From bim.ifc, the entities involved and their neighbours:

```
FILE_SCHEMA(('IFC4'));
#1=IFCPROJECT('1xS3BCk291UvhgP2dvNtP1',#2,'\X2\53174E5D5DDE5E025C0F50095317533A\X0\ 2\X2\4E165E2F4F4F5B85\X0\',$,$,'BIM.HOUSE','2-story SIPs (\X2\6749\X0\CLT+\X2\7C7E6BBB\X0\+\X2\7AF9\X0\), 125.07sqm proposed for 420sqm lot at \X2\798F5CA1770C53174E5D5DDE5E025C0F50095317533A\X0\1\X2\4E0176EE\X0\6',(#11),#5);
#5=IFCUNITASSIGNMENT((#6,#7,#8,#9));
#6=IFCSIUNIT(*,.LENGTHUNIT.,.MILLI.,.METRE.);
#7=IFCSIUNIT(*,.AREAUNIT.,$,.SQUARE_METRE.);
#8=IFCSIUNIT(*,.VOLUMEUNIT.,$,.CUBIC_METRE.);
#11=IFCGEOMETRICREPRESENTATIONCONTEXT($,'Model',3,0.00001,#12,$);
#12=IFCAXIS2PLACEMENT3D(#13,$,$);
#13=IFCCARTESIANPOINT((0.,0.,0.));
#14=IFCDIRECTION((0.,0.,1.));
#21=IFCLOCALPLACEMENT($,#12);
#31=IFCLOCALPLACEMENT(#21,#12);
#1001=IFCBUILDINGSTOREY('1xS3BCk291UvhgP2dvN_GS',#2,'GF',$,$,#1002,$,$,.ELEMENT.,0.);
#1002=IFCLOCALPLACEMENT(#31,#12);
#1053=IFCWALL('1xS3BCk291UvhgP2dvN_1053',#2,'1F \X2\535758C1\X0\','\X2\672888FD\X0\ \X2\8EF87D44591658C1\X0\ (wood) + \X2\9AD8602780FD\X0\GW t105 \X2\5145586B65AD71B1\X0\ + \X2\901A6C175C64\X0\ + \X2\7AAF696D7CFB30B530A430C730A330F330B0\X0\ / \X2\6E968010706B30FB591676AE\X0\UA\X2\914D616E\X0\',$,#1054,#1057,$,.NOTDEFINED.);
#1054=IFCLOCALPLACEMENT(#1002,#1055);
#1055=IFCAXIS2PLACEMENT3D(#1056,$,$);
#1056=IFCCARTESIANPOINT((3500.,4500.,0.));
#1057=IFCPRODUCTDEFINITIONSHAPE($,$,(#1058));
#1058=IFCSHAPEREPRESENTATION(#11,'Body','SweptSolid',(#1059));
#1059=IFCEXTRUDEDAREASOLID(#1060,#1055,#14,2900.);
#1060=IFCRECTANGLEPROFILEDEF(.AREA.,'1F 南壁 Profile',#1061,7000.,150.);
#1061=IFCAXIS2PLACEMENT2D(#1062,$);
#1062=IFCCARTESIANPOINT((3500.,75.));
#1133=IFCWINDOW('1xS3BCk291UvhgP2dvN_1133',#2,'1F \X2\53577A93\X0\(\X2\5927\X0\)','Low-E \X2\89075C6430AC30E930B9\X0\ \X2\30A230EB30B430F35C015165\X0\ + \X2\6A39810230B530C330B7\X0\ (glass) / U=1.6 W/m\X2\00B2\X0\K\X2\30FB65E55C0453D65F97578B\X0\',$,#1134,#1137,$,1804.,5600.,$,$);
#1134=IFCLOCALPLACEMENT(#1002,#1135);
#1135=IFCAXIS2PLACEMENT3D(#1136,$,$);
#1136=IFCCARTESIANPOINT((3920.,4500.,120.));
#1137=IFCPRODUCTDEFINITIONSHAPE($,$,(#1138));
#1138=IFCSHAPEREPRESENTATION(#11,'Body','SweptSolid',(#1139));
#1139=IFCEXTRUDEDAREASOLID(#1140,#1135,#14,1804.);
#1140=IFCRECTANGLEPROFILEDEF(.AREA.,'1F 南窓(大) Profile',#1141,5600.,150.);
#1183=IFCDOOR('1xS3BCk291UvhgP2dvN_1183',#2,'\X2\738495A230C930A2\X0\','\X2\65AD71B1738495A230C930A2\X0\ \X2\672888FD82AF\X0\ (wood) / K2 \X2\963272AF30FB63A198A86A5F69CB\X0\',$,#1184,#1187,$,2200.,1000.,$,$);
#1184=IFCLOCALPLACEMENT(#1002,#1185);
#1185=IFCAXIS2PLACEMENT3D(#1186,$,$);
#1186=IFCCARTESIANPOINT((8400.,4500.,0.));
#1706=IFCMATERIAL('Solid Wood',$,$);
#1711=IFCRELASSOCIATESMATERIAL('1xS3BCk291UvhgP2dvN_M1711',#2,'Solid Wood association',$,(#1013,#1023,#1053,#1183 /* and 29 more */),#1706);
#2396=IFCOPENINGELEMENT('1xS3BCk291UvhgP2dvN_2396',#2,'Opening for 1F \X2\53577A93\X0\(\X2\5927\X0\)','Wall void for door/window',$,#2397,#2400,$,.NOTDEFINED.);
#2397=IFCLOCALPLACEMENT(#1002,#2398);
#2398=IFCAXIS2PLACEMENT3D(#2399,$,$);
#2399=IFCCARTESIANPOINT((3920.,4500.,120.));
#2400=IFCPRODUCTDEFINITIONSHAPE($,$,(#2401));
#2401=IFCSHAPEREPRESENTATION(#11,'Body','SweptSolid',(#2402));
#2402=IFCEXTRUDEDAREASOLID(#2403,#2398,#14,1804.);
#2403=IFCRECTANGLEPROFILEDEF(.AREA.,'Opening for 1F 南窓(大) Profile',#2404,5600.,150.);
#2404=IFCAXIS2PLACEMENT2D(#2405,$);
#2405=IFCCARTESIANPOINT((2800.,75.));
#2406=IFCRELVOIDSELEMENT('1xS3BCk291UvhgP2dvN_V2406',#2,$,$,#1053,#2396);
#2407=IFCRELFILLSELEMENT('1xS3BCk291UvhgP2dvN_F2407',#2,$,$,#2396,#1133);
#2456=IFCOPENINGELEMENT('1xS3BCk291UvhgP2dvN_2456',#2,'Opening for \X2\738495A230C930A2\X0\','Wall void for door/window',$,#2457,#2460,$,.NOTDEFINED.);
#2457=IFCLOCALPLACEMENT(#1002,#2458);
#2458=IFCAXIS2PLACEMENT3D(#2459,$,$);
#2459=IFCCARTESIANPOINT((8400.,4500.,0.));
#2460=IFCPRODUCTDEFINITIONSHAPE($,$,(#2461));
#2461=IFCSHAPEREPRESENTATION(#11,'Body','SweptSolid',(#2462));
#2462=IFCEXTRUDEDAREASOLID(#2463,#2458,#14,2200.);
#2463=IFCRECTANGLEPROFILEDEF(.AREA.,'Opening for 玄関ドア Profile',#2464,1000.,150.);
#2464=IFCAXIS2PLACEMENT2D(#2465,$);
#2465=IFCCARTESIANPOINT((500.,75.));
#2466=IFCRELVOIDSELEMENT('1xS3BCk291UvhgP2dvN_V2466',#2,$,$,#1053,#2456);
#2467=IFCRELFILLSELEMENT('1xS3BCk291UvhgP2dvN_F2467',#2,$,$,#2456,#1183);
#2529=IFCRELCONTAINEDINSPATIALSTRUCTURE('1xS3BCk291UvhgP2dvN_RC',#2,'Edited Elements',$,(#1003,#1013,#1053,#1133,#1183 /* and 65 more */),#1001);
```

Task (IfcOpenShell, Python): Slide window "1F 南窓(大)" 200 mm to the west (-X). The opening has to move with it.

```python
import ifcopenshell
import ifcopenshell.api.geometry
import ifcopenshell.util.placement

model = ifcopenshell.open("bim.ifc")

window = model.by_guid("1xS3BCk291UvhgP2dvN_1133")
opening = window.FillsVoids[0].RelatingOpeningElement
wall = opening.VoidsElements[0].RelatingBuildingElement

wall_matrix = ifcopenshell.util.placement.get_local_placement(wall.ObjectPlacement)
shift = wall_matrix[:3, 0] * -200.0
before = ifcopenshell.util.placement.get_local_placement(window.ObjectPlacement)[:3, 3].copy()

# The window is not placed relative to its opening, so move both.
for product in (opening, window):
    matrix = ifcopenshell.util.placement.get_local_placement(product.ObjectPlacement)
    matrix[:3, 3] += shift
    ifcopenshell.api.geometry.edit_object_placement(model, product=product, matrix=matrix, is_si=False)

after = ifcopenshell.util.placement.get_local_placement(window.ObjectPlacement)[:3, 3]
print("window moved by", (after - before).round(3) + 0.0)

model.write("bim_v2.ifc")
```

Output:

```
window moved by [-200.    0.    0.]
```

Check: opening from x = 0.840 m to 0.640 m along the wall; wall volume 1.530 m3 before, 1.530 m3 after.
